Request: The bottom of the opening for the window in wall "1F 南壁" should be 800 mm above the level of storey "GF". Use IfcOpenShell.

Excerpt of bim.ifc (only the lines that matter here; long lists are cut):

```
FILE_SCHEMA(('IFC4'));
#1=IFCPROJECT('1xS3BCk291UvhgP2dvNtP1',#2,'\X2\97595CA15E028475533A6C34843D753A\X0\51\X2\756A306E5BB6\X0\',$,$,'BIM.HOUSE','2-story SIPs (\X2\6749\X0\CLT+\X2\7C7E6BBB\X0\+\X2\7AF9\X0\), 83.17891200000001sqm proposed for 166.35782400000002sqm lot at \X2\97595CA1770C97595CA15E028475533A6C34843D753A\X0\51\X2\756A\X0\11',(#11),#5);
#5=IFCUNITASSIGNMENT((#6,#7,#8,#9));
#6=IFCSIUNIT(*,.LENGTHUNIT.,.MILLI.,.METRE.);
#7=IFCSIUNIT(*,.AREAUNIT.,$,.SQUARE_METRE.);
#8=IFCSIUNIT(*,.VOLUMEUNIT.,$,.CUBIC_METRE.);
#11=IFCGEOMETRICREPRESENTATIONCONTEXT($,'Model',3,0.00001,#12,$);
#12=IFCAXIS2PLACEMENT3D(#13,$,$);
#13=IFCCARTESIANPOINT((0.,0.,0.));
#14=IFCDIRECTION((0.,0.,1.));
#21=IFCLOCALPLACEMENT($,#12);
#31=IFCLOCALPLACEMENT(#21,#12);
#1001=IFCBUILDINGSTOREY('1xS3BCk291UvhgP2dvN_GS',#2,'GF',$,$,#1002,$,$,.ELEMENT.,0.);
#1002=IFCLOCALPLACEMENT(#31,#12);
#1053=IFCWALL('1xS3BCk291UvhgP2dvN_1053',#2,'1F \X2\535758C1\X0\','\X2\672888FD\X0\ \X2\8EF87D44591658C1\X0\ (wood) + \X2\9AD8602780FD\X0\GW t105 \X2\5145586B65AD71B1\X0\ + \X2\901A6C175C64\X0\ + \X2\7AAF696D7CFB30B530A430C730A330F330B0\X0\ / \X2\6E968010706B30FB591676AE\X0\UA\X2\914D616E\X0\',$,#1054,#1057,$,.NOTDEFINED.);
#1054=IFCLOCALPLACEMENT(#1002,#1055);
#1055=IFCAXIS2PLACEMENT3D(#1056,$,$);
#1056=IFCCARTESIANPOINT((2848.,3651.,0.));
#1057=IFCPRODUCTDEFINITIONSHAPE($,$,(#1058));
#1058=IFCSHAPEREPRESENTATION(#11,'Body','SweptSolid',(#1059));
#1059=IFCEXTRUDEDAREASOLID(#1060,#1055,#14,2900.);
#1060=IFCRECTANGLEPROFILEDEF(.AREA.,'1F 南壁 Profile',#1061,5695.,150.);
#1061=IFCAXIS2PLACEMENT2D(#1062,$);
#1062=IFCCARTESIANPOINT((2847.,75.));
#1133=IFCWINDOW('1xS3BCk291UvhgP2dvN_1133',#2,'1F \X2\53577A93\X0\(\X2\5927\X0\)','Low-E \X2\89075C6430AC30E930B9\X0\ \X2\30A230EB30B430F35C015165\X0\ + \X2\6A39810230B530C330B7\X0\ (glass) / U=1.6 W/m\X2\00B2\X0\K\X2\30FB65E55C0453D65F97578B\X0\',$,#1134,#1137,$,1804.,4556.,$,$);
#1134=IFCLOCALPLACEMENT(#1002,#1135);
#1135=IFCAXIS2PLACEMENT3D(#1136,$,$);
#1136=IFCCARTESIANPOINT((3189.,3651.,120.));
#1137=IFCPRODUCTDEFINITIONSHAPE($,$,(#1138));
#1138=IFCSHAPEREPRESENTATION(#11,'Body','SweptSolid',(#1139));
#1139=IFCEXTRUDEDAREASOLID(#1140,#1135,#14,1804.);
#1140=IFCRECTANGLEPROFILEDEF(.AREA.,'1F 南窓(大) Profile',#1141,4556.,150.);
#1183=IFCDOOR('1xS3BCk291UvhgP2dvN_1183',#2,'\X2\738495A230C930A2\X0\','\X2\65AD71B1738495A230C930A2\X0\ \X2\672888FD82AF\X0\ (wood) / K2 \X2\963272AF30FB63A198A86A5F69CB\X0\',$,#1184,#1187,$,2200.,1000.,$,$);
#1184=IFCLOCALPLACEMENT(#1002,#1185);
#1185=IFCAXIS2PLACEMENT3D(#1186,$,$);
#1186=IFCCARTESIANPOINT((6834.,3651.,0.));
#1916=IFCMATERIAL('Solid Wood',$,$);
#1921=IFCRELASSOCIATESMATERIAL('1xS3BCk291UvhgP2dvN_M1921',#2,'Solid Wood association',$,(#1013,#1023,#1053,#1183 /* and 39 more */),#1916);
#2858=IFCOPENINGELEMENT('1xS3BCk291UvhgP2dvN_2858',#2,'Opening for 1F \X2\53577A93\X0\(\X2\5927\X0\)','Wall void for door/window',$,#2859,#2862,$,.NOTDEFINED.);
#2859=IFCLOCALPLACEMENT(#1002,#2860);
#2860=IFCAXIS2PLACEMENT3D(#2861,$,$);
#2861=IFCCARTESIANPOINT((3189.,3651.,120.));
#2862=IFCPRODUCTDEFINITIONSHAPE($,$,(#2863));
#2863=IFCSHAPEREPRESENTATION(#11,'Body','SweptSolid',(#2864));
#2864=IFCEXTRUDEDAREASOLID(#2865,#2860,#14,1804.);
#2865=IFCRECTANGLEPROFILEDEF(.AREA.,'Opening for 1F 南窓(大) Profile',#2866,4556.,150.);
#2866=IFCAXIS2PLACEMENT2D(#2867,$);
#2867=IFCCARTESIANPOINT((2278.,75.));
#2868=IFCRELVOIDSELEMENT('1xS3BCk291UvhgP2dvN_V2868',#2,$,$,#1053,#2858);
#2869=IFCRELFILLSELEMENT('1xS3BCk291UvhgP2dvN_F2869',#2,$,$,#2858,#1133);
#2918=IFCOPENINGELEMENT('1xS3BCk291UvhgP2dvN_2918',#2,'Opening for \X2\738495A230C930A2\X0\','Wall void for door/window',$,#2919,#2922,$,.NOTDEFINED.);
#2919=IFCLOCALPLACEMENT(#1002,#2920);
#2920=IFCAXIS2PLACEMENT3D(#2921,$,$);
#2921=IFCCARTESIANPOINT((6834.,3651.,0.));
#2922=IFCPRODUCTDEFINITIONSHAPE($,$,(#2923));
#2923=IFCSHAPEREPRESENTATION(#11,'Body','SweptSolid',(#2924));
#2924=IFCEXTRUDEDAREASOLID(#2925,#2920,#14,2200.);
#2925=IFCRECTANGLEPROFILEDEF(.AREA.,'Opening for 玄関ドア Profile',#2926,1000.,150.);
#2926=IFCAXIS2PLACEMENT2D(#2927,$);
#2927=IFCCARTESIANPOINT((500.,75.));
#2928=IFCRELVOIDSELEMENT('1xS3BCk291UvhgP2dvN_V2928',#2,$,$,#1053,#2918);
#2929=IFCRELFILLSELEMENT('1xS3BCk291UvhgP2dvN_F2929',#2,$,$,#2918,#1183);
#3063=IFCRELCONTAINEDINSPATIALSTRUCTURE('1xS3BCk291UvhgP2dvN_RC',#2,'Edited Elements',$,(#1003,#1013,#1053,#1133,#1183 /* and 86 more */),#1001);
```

```python
import numpy as np
import ifcopenshell
import ifcopenshell.api.geometry
import ifcopenshell.geom
import ifcopenshell.util.element
import ifcopenshell.util.placement
import ifcopenshell.util.shape
import ifcopenshell.util.unit

model = ifcopenshell.open("bim.ifc")
unit_scale = ifcopenshell.util.unit.calculate_unit_scale(model)

window = model.by_guid("1xS3BCk291UvhgP2dvN_1133")
opening = window.FillsVoids[0].RelatingOpeningElement
storey = ifcopenshell.util.element.get_container(window, ifc_class="IfcBuildingStorey")
level = ifcopenshell.util.placement.get_local_placement(storey.ObjectPlacement)[2, 3]

# The opening's origin need not be at the sill, so measure its lowest point.
shape = ifcopenshell.geom.create_shape(ifcopenshell.geom.settings(), opening)
bottom = ifcopenshell.util.shape.get_shape_bottom_elevation(shape, shape.geometry) / unit_scale
dz = level + 800.0 - bottom

shift = np.array([0.0, 0.0, dz])
# The window is not placed relative to its opening, so move both.
for product in (opening, window):
    matrix = ifcopenshell.util.placement.get_local_placement(product.ObjectPlacement)
    matrix[:3, 3] += shift
    ifcopenshell.api.geometry.edit_object_placement(model, product=product, matrix=matrix, is_si=False)

print(f"moved by {dz * unit_scale:+.3f} m")

model.write("bim_updated.ifc")
```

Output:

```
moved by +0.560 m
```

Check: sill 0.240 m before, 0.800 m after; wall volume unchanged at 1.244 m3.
